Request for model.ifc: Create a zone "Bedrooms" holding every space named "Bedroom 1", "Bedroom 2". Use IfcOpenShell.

First a look at what the model holds.

```python
import ifcopenshell

model = ifcopenshell.open("model.ifc")
print(model.schema)
seen = {}
for space in model.by_type("IfcSpace"):
    seen[space.LongName] = seen.get(space.LongName, 0) + 1
for name, count in sorted(seen.items(), key=str):
    print(count, "x", name)
print("zones:", [z.Name for z in model.by_type("IfcZone")][:20])
```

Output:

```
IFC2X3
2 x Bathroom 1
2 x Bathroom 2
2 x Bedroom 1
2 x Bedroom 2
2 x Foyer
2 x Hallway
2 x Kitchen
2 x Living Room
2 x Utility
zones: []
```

```python
import ifcopenshell
import ifcopenshell.api.group
import ifcopenshell.api.root

model = ifcopenshell.open("model.ifc")

names = {"Bedroom 1", "Bedroom 2"}
spaces = [s for s in model.by_type("IfcSpace") if s.LongName in names]

zone = ifcopenshell.api.root.create_entity(model, ifc_class="IfcZone", name="Bedrooms")
ifcopenshell.api.group.assign_group(model, products=spaces, group=zone)
print(len(spaces), "spaces in", zone.Name)

model.write("model-out.ifc")
```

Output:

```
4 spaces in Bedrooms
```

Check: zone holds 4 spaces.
